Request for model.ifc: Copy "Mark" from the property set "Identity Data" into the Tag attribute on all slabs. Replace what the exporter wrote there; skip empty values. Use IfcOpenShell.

First a look at what the model holds.

```python
import ifcopenshell
import ifcopenshell.util.element

model = ifcopenshell.open("model.ifc")
print(model.schema)
slabs = model.by_type("IfcSlab")
print(len(slabs), "slabs")
for e in slabs[:8]:
    source = ifcopenshell.util.element.get_pset(e, "Identity Data", "Mark")
    target = e.Tag
    print(e.id(), repr(source), repr(target), sep=" | ")
```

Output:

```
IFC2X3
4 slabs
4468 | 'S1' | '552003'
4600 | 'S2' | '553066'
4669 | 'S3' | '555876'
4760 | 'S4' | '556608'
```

```python
import ifcopenshell
import ifcopenshell.util.element

model = ifcopenshell.open("model.ifc")

count = 0
for e in model.by_type("IfcSlab"):
    value = ifcopenshell.util.element.get_pset(e, "Identity Data", "Mark")
    current = e.Tag
    if not value or not value.strip() or current == value:
        continue
    e.Tag = value
    count += 1

print(count, "slabs updated")

model.write("model_edited.ifc")
```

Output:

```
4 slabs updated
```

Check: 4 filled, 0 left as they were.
